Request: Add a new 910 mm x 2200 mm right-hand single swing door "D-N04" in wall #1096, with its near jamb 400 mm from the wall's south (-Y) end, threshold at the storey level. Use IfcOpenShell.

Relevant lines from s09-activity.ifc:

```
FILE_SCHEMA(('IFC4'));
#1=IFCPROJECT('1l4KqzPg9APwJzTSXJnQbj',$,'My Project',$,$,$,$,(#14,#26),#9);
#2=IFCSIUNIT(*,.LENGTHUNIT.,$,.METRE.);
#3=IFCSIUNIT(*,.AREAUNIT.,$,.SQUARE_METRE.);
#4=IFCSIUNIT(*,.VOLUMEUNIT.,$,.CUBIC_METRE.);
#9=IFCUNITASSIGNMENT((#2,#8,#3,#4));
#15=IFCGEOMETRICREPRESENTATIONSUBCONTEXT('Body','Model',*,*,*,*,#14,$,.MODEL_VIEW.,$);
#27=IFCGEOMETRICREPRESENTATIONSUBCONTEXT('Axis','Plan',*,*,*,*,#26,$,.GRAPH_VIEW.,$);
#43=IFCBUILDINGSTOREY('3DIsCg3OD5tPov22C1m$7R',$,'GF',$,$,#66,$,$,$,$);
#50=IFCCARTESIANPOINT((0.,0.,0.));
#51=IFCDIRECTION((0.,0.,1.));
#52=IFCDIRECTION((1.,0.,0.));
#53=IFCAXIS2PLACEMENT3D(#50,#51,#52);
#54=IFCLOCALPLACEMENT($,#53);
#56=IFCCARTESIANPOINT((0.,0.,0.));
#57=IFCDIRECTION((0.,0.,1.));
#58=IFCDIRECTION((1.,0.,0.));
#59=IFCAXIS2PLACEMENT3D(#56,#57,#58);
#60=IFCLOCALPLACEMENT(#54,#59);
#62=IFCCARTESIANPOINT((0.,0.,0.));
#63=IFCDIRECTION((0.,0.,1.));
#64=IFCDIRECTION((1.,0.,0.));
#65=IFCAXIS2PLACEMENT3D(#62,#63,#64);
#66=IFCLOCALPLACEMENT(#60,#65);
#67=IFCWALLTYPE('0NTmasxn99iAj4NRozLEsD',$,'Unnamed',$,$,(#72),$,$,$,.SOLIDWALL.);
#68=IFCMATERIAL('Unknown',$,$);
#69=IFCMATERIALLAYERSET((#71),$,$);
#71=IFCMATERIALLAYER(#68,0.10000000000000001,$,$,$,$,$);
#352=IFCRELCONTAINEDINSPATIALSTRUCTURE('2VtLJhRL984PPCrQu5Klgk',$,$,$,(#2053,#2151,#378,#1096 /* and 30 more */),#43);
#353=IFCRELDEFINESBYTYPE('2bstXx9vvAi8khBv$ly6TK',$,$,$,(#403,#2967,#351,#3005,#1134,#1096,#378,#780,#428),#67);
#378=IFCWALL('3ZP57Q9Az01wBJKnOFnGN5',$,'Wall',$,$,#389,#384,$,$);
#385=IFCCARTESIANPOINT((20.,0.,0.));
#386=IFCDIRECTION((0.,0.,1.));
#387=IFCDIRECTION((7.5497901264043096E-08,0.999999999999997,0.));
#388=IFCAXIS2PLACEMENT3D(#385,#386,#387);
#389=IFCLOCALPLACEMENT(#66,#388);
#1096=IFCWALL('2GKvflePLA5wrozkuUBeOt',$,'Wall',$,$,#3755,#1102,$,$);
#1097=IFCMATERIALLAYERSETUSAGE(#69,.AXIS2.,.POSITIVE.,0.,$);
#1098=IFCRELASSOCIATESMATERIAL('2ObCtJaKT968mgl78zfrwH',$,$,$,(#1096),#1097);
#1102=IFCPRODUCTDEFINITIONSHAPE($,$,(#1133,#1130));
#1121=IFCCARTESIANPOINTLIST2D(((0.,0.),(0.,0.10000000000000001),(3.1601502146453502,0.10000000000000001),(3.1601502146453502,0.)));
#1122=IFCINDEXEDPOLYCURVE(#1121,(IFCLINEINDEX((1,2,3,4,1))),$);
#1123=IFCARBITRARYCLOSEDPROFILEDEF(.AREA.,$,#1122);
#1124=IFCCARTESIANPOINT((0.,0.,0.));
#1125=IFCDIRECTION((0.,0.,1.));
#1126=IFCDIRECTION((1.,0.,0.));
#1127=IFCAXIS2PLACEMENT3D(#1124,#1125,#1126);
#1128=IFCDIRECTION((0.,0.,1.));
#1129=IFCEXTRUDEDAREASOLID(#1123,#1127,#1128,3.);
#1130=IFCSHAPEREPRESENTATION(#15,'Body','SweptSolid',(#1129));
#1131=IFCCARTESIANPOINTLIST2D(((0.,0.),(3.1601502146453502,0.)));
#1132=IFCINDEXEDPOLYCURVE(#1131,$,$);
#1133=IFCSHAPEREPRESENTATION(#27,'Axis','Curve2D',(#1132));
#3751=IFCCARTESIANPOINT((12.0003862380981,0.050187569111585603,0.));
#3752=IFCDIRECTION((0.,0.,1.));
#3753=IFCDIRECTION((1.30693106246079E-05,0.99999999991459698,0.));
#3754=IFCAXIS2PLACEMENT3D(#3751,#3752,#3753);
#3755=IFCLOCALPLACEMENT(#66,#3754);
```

```python
import numpy as np
import ifcopenshell
import ifcopenshell.api.feature
import ifcopenshell.api.geometry
import ifcopenshell.api.root
import ifcopenshell.api.spatial
import ifcopenshell.geom
import ifcopenshell.util.element
import ifcopenshell.util.placement
import ifcopenshell.util.representation
import ifcopenshell.util.shape
import ifcopenshell.util.unit

model = ifcopenshell.open("s09-activity.ifc")
unit_scale = ifcopenshell.util.unit.calculate_unit_scale(model)
settings = ifcopenshell.geom.settings()


def volume(element):
    """Net volume in cubic metres, openings subtracted."""
    shape = ifcopenshell.geom.create_shape(settings, element)
    return ifcopenshell.util.shape.get_volume(shape.geometry)


wall = model.by_guid("2GKvflePLA5wrozkuUBeOt")
storey = ifcopenshell.util.element.get_container(wall, ifc_class="IfcBuildingStorey")
context = ifcopenshell.util.representation.get_context(model, "Model", "Body", "MODEL_VIEW")
before = volume(wall)

width, height, from_end, sill = 0.91, 2.2, 0.4, 0.0  # metres

# The wall runs along its own X axis, and the end named is its -X end.
wall_shape = ifcopenshell.geom.create_shape(settings, wall)
x, y, z = ifcopenshell.util.shape.get_vertices(wall_shape.geometry).T
start = x.min() + from_end
face, thickness = float(y.min()), float(y.max() - y.min())
wall_matrix = ifcopenshell.util.placement.get_local_placement(wall.ObjectPlacement)
level = ifcopenshell.util.placement.get_local_placement(storey.ObjectPlacement)[2, 3]


def in_wall(x, y):
    """Placement at x, y metres in the wall's axes, at sill height."""
    matrix = wall_matrix.copy()
    matrix[:, 3] = wall_matrix @ np.array([x / unit_scale, y / unit_scale, 0.0, 1.0])
    matrix[2, 3] = level + sill / unit_scale
    return matrix


# Opening: a box that overshoots both wall faces by 50 mm.
opening = ifcopenshell.api.root.create_entity(model, ifc_class="IfcOpeningElement", predefined_type="OPENING")
box = ifcopenshell.api.geometry.add_wall_representation(
    model, context=context, length=width, height=height, thickness=thickness + 0.1
)
ifcopenshell.api.geometry.assign_representation(model, product=opening, representation=box)
ifcopenshell.api.geometry.edit_object_placement(model, product=opening, matrix=in_wall(start, face - 0.05), is_si=False)
ifcopenshell.api.feature.add_feature(model, feature=opening, element=wall)

door = ifcopenshell.api.root.create_entity(model, ifc_class="IfcDoor", name="D-N04", predefined_type="DOOR")
door.OverallWidth, door.OverallHeight = width / unit_scale, height / unit_scale
door.OperationType = "SINGLE_SWING_RIGHT"
body = ifcopenshell.api.geometry.add_door_representation(
    model,
    context=context,
    overall_width=door.OverallWidth,
    overall_height=door.OverallHeight,
    operation_type="SINGLE_SWING_RIGHT",
    lining_properties={"LiningDepth": thickness / unit_scale, "ThresholdDepth": thickness / unit_scale},
)
ifcopenshell.api.geometry.assign_representation(model, product=door, representation=body)
ifcopenshell.api.spatial.assign_container(model, products=[door], relating_structure=storey)
ifcopenshell.api.feature.add_filling(model, opening=opening, element=door)

# The lining spans the wall, so the door starts at the wall face.
ifcopenshell.api.geometry.edit_object_placement(model, product=door, matrix=in_wall(start, face), is_si=False)

after = volume(wall)

print(f"wall volume {before:.3f} -> {after:.3f} m3")

model.write("s09-activity_edited.ifc")
```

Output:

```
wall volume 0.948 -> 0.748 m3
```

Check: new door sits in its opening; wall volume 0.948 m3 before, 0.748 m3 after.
